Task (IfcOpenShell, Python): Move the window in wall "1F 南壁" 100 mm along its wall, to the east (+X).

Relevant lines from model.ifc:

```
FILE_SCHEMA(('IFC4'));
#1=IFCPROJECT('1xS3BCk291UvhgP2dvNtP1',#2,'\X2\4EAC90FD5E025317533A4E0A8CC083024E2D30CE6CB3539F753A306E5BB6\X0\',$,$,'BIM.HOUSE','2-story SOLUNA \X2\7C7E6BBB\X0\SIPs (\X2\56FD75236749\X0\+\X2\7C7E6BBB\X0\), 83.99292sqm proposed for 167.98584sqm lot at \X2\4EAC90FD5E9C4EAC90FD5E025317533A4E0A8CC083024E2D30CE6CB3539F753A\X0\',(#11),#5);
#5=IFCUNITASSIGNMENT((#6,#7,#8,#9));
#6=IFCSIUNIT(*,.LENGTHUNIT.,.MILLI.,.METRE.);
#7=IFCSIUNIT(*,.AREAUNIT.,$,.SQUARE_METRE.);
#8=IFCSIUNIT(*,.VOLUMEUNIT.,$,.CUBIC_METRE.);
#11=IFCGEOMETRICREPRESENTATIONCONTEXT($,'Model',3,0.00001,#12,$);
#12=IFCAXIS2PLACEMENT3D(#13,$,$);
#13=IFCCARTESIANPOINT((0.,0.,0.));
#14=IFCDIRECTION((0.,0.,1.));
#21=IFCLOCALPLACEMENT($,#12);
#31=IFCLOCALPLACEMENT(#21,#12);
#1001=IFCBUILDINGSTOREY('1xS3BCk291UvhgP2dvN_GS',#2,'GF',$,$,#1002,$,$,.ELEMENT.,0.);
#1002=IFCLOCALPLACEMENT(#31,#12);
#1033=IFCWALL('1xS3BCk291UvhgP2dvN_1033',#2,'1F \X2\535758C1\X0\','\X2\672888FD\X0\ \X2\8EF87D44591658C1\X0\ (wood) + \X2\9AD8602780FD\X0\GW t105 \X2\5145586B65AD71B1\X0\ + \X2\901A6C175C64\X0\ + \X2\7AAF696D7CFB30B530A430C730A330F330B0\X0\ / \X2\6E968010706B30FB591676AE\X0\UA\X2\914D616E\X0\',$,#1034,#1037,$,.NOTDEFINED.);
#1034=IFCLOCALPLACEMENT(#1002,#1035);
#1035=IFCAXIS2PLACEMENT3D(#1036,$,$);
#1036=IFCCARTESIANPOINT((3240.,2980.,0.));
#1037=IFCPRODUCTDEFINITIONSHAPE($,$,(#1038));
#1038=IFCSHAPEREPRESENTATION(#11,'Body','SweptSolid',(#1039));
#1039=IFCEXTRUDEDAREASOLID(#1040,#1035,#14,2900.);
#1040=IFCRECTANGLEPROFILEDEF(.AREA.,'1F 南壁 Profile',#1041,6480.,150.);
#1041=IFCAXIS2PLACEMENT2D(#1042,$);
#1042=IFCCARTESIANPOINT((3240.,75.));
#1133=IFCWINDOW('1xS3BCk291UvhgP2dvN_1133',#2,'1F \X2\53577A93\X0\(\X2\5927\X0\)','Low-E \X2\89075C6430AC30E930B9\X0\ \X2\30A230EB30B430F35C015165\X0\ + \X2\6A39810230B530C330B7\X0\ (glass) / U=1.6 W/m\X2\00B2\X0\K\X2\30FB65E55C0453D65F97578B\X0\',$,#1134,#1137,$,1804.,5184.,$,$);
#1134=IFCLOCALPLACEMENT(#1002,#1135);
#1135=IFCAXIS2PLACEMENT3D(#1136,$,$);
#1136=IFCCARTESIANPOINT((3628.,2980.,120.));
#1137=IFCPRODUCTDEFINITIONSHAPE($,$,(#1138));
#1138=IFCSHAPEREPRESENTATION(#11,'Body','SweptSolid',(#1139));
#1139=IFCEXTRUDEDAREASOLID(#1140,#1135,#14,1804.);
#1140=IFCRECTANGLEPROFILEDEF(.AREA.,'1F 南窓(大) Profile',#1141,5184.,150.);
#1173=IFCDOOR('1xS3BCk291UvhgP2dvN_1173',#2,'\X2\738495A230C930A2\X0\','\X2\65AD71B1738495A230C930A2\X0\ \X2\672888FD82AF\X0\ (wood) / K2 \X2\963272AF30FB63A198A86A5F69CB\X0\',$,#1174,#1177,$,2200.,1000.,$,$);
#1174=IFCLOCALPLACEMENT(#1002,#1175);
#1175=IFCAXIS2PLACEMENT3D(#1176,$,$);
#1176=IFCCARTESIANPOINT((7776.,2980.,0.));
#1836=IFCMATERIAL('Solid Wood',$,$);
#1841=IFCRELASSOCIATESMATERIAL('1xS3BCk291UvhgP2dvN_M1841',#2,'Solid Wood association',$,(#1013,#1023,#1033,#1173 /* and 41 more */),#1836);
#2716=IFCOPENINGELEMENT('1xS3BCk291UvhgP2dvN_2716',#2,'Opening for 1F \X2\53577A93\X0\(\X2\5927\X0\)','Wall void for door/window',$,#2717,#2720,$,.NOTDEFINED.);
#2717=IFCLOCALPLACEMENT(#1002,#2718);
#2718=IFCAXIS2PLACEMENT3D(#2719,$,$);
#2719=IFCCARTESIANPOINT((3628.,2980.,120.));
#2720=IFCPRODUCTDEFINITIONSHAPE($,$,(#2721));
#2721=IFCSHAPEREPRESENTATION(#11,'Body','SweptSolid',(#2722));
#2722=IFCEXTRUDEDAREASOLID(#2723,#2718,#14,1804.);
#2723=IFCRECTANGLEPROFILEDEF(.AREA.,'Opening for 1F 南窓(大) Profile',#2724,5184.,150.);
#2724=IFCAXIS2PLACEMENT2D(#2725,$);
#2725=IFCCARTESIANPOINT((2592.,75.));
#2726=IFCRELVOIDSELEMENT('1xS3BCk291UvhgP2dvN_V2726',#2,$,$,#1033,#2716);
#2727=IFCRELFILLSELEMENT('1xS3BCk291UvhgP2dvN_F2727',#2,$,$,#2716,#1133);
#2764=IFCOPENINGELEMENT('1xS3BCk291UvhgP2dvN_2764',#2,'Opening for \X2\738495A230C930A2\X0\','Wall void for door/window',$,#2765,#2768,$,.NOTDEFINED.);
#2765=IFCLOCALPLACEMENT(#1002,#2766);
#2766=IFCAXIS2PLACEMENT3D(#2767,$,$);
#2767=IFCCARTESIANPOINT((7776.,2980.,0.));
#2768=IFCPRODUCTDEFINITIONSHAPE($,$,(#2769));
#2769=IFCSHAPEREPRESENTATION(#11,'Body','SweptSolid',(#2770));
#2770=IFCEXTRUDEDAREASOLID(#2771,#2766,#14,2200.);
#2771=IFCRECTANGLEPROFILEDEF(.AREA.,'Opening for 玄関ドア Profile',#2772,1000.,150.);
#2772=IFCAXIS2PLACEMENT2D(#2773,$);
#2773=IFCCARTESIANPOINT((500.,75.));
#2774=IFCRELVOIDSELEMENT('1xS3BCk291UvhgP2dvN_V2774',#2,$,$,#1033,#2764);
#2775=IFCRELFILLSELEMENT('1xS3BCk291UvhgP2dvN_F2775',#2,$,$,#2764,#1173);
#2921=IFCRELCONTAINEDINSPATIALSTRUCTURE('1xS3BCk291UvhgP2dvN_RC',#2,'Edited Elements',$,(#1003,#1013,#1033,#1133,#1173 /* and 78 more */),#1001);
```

```python
import ifcopenshell
import ifcopenshell.api.geometry
import ifcopenshell.util.placement
import ifcopenshell.util.unit

model = ifcopenshell.open("model.ifc")
unit_scale = ifcopenshell.util.unit.calculate_unit_scale(model)

window = model.by_guid("1xS3BCk291UvhgP2dvN_1133")
opening = window.FillsVoids[0].RelatingOpeningElement
wall = opening.VoidsElements[0].RelatingBuildingElement

wall_matrix = ifcopenshell.util.placement.get_local_placement(wall.ObjectPlacement)
shift = wall_matrix[:3, 0] * 0.1 / unit_scale
before = ifcopenshell.util.placement.get_local_placement(window.ObjectPlacement)[:3, 3].copy()

# The window is not placed relative to its opening, so move both.
for product in (opening, window):
    matrix = ifcopenshell.util.placement.get_local_placement(product.ObjectPlacement)
    matrix[:3, 3] += shift
    ifcopenshell.api.geometry.edit_object_placement(model, product=product, matrix=matrix, is_si=False)

after = ifcopenshell.util.placement.get_local_placement(window.ObjectPlacement)[:3, 3]
print("window moved by", (after - before).round(3) + 0.0)

model.write("model_v2.ifc")
```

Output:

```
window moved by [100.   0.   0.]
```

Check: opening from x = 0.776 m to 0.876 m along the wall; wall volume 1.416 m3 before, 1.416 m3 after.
